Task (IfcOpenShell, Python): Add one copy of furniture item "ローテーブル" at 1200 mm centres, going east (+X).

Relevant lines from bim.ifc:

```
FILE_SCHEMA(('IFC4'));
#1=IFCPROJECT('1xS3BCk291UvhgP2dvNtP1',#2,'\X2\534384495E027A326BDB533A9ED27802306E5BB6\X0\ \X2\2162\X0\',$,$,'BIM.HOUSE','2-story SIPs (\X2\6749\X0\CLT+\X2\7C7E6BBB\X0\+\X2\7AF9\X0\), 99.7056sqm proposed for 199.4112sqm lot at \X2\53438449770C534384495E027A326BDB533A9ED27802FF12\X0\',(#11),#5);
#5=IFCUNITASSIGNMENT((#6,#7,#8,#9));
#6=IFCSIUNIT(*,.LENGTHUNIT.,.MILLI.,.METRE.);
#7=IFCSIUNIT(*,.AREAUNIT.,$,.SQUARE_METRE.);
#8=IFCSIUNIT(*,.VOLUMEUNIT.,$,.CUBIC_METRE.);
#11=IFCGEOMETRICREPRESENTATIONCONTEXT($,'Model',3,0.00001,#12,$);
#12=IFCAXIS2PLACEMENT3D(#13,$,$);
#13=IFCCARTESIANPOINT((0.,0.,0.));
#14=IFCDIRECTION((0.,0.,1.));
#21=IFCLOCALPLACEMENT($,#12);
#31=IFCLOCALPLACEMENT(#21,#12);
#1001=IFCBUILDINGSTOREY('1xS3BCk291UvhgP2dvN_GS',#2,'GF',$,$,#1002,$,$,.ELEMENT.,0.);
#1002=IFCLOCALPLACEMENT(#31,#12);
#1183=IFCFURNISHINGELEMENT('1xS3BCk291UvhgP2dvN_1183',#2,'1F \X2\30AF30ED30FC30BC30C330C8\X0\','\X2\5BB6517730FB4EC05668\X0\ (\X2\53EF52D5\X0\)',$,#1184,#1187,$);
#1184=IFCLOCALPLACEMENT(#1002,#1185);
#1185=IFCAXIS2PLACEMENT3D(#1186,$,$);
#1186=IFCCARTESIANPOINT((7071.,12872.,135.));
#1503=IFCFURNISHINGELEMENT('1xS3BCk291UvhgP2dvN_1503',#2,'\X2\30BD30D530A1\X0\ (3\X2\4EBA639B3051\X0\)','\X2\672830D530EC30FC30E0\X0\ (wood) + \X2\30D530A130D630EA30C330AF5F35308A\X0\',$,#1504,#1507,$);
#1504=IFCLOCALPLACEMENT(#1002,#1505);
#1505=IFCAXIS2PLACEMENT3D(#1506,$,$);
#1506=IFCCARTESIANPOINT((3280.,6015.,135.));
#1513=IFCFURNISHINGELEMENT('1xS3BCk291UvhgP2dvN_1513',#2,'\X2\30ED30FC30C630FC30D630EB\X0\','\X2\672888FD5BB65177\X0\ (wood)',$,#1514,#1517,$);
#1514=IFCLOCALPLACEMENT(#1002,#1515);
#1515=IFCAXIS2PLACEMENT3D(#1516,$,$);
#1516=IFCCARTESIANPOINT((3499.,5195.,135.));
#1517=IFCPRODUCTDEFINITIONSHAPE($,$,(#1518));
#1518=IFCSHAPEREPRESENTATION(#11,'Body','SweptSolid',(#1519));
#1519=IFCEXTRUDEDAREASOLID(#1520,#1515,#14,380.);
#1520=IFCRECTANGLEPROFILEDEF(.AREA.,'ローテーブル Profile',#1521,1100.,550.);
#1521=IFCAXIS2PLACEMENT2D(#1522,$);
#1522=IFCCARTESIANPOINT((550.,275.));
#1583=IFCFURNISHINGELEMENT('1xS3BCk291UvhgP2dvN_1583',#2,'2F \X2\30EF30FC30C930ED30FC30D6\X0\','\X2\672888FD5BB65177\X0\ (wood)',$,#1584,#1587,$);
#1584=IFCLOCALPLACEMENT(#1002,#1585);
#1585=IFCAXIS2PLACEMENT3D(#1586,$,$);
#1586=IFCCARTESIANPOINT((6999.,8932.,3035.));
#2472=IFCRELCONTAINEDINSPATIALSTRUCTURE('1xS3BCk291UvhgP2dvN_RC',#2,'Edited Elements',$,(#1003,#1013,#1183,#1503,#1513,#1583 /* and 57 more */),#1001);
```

```python
import numpy as np
import ifcopenshell
import ifcopenshell.api.geometry
import ifcopenshell.api.root
import ifcopenshell.util.element
import ifcopenshell.util.placement
import ifcopenshell.util.unit

model = ifcopenshell.open("bim.ifc")
unit_scale = ifcopenshell.util.unit.calculate_unit_scale(model)


def reuse_history(source, copy):
    """copy_class also copies each property set's owner history, people and application; keep the originals."""
    for rel in copy.IsDefinedBy:
        if rel.is_a("IfcRelDefinesByProperties") and (history := rel.RelatingPropertyDefinition.OwnerHistory):
            rel.RelatingPropertyDefinition.OwnerHistory = source.OwnerHistory
            ifcopenshell.util.element.remove_deep2(model, history)


source = model.by_id(1513)
base = ifcopenshell.util.placement.get_local_placement(source.ObjectPlacement)
step = np.array([1.0, 0.0, 0.0]) * 1.2 / unit_scale

for i in range(1, 2):
    copy = ifcopenshell.api.root.copy_class(model, product=source)
    copy.Representation = ifcopenshell.util.element.copy_deep(
        model, source.Representation, exclude=["IfcGeometricRepresentationContext", "IfcRepresentationMap"]
    )
    reuse_history(source, copy)
    matrix = base.copy()
    matrix[:3, 3] += i * step
    print("added at", matrix[:3, 3].round(3) + 0.0)
    ifcopenshell.api.geometry.edit_object_placement(model, product=copy, matrix=matrix, is_si=False)

model.write("bim_edited.ifc")
```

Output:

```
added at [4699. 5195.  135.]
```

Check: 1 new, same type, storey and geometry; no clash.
